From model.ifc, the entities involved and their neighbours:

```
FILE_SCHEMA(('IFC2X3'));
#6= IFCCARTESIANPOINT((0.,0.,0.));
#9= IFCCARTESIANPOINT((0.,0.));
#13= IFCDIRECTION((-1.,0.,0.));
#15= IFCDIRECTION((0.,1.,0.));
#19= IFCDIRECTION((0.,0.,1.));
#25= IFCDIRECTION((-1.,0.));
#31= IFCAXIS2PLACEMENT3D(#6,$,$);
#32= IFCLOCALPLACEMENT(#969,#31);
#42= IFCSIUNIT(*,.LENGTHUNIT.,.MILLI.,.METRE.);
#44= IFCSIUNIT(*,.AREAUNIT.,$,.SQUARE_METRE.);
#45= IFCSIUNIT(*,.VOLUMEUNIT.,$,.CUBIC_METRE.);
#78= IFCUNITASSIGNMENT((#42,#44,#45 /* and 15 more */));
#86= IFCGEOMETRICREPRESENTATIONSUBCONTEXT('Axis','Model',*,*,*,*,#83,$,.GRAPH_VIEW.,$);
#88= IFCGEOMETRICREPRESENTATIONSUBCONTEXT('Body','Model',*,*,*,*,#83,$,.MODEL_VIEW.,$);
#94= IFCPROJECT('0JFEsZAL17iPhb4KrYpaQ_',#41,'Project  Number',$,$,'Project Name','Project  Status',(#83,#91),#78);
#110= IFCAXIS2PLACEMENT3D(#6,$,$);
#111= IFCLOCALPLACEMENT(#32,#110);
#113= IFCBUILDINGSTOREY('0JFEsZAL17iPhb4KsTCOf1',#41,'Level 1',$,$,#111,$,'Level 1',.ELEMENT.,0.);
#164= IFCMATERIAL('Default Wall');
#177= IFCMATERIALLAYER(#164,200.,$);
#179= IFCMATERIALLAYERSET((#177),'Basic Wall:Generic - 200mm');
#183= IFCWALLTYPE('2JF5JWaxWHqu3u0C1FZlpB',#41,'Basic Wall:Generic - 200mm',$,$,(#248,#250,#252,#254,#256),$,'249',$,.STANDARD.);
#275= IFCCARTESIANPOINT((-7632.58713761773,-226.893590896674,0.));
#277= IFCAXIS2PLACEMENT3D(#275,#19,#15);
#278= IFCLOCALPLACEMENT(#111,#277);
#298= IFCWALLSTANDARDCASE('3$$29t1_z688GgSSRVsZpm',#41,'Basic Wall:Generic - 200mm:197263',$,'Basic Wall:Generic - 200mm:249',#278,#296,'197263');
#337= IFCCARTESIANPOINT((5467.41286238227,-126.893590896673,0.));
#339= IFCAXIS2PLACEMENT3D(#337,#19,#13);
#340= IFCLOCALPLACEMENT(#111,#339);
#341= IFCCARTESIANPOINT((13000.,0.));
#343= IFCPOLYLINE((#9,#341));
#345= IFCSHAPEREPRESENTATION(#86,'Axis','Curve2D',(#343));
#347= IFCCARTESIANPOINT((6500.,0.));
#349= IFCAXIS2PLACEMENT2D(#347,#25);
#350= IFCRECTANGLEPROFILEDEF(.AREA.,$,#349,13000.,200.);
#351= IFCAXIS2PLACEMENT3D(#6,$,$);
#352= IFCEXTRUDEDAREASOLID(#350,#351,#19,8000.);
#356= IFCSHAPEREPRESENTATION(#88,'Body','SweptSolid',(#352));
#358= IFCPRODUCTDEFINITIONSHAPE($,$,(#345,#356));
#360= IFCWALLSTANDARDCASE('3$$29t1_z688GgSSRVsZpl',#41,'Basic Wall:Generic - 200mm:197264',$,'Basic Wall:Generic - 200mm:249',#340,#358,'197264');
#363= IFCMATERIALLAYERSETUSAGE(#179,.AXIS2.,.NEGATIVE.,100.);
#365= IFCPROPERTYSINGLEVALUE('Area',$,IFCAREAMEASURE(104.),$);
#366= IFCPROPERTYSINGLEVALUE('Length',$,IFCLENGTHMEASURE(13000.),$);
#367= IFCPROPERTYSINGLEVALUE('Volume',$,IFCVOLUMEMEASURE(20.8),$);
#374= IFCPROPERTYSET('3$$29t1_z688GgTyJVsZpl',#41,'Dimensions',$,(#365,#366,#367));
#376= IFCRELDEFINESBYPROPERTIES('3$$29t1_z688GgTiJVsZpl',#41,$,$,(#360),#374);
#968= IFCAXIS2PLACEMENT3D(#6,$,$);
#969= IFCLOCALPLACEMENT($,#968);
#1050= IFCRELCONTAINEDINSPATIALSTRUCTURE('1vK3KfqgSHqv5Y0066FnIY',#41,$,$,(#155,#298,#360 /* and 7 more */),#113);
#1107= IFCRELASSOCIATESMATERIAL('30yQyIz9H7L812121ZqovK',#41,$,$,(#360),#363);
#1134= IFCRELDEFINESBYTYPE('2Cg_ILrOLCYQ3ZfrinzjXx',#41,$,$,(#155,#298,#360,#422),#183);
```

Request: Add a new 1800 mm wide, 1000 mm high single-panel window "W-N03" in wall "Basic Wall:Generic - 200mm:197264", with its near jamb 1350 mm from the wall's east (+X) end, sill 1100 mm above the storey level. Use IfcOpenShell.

```python
import numpy as np
import ifcopenshell
import ifcopenshell.api.feature
import ifcopenshell.api.geometry
import ifcopenshell.api.pset
import ifcopenshell.api.root
import ifcopenshell.api.spatial
import ifcopenshell.api.type
import ifcopenshell.geom
import ifcopenshell.util.element
import ifcopenshell.util.placement
import ifcopenshell.util.representation
import ifcopenshell.util.shape
import ifcopenshell.util.unit

model = ifcopenshell.open("model.ifc")
unit_scale = ifcopenshell.util.unit.calculate_unit_scale(model)
area_scale = ifcopenshell.util.unit.calculate_unit_scale(model, "AREAUNIT")
volume_scale = ifcopenshell.util.unit.calculate_unit_scale(model, "VOLUMEUNIT")
settings = ifcopenshell.geom.settings()


def volume(element):
    """Net volume in cubic metres, openings subtracted."""
    shape = ifcopenshell.geom.create_shape(settings, element)
    return ifcopenshell.util.shape.get_volume(shape.geometry)


wall = model.by_id(360)
storey = ifcopenshell.util.element.get_container(wall, ifc_class="IfcBuildingStorey")
context = ifcopenshell.util.representation.get_context(model, "Model", "Body", "MODEL_VIEW")
before = volume(wall)

width, height, from_end, sill = 1.8, 1, 1.35, 1.1  # metres

# The wall runs along its own X axis, and the end named is its -X end.
wall_shape = ifcopenshell.geom.create_shape(settings, wall)
x, y, z = ifcopenshell.util.shape.get_vertices(wall_shape.geometry).T
start = x.min() + from_end
face, thickness = float(y.min()), float(y.max() - y.min())
wall_matrix = ifcopenshell.util.placement.get_local_placement(wall.ObjectPlacement)
level = ifcopenshell.util.placement.get_local_placement(storey.ObjectPlacement)[2, 3]


def in_wall(x, y):
    """Placement at x, y metres in the wall's axes, at sill height."""
    matrix = wall_matrix.copy()
    matrix[:, 3] = wall_matrix @ np.array([x / unit_scale, y / unit_scale, 0.0, 1.0])
    matrix[2, 3] = level + sill / unit_scale
    return matrix


# Opening: a box that overshoots both wall faces by 50 mm.
opening = ifcopenshell.api.root.create_entity(model, ifc_class="IfcOpeningElement")
box = ifcopenshell.api.geometry.add_wall_representation(
    model, context=context, length=width, height=height, thickness=thickness + 0.1
)
ifcopenshell.api.geometry.assign_representation(model, product=opening, representation=box)
ifcopenshell.api.geometry.edit_object_placement(model, product=opening, matrix=in_wall(start, face - 0.05), is_si=False)
ifcopenshell.api.feature.add_feature(model, feature=opening, element=wall)

window = ifcopenshell.api.root.create_entity(model, ifc_class="IfcWindow", name="W-N03")
window.OverallWidth, window.OverallHeight = width / unit_scale, height / unit_scale
body = ifcopenshell.api.geometry.add_window_representation(
    model,
    context=context,
    overall_width=window.OverallWidth,
    overall_height=window.OverallHeight,
    partition_type="SINGLE_PANEL",
)
ifcopenshell.api.geometry.assign_representation(model, product=window, representation=body)
ifcopenshell.api.spatial.assign_container(model, products=[window], relating_structure=storey)
fills = ifcopenshell.api.feature.add_filling(model, opening=opening, element=window)
fills.OwnerHistory = window.OwnerHistory  # required in IFC2X3

# IFC2X3 keeps the operation on the window style.
style = ifcopenshell.api.root.create_entity(model, ifc_class="IfcWindowStyle", name="W-N03")
style.OperationType, style.ConstructionType = "SINGLE_PANEL", "NOTDEFINED"
style.ParameterTakesPrecedence = style.Sizeable = False
ifcopenshell.api.type.assign_type(model, related_objects=[window], relating_type=style)

# Centre the window in the wall's thickness.
ifcopenshell.api.geometry.edit_object_placement(model, product=window, matrix=in_wall(start, face), is_si=False)
window_shape = ifcopenshell.geom.create_shape(settings, window)
depth = ifcopenshell.util.shape.get_vertices(window_shape.geometry)[:, 1]
offset = face + thickness / 2 - (depth.min() + depth.max()) / 2
ifcopenshell.api.geometry.edit_object_placement(model, product=window, matrix=in_wall(start, offset), is_si=False)

after = volume(wall)

# Update the wall's stored quantities.
pset = model.by_id(ifcopenshell.util.element.get_pset(wall, "Dimensions", should_inherit=False)["id"])
ifcopenshell.api.pset.edit_pset(model, pset=pset, properties={
    "Area": model.create_entity("IfcAreaMeasure", after / thickness / area_scale),
    "Volume": model.create_entity("IfcVolumeMeasure", after / volume_scale),
})

print(f"wall volume {before:.3f} -> {after:.3f} m3")

model.write("model_updated.ifc")
```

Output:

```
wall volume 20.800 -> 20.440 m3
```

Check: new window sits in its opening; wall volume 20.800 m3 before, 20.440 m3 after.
